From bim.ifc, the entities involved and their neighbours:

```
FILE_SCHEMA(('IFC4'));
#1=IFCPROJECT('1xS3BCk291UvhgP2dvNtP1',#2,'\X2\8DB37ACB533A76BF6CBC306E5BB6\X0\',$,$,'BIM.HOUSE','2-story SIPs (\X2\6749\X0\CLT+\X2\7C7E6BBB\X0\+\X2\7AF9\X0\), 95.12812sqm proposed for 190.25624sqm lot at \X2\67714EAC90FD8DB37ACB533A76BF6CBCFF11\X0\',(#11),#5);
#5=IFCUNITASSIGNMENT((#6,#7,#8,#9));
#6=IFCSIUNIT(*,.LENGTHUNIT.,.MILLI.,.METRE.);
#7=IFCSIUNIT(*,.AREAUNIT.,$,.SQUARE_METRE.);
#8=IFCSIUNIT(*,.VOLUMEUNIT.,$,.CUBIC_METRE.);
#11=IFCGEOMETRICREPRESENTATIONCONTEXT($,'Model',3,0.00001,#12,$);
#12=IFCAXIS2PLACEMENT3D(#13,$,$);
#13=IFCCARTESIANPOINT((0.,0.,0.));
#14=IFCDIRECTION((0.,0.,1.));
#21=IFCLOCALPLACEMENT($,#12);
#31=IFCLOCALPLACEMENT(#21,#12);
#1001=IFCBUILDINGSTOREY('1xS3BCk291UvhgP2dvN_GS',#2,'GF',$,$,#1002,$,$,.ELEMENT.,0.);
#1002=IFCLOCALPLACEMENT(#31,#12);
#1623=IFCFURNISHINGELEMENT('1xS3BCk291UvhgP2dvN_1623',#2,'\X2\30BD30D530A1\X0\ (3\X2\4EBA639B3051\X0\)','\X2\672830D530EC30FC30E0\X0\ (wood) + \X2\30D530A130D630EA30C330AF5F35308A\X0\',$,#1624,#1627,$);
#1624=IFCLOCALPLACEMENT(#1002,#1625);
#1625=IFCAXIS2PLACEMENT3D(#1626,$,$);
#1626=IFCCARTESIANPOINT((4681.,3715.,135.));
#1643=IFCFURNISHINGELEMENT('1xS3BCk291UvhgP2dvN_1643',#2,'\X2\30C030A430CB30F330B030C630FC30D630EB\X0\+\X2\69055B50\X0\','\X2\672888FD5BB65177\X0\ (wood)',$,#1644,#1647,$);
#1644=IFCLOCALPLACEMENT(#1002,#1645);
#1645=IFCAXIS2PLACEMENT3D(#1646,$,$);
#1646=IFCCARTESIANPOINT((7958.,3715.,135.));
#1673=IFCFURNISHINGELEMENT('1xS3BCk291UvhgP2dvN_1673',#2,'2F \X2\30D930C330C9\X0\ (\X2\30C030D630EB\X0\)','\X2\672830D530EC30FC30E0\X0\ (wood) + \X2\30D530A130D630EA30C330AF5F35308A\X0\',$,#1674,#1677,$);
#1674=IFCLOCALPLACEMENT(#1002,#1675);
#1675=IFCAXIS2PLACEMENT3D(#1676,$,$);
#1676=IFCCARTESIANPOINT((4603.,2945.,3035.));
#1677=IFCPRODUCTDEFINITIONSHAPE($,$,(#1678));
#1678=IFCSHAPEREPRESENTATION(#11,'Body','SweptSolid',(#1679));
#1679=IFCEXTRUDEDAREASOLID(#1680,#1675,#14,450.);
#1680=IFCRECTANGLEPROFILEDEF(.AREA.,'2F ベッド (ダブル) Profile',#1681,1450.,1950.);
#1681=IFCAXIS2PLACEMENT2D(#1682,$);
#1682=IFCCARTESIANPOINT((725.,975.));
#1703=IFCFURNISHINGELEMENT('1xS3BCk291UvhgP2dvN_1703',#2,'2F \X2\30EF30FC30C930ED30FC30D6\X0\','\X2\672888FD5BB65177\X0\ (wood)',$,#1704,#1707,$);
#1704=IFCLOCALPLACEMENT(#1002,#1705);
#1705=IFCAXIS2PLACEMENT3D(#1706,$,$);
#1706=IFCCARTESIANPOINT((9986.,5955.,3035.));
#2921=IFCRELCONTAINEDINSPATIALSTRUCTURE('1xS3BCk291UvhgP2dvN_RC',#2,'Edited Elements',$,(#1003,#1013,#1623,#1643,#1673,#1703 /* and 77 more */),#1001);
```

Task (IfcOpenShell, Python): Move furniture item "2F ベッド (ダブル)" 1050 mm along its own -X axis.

```python
import ifcopenshell
import ifcopenshell.api.geometry
import ifcopenshell.util.placement
import ifcopenshell.util.unit

model = ifcopenshell.open("bim.ifc")
unit_scale = ifcopenshell.util.unit.calculate_unit_scale(model)

item = model.by_id(1673)
matrix = ifcopenshell.util.placement.get_local_placement(item.ObjectPlacement)
matrix[:3, 3] -= matrix[:3, 0] * 1.05 / unit_scale
ifcopenshell.api.geometry.edit_object_placement(model, product=item, matrix=matrix, is_si=False)

print(ifcopenshell.util.placement.get_local_placement(item.ObjectPlacement).round(3) + 0.0)

model.write("bim-out.ifc")
```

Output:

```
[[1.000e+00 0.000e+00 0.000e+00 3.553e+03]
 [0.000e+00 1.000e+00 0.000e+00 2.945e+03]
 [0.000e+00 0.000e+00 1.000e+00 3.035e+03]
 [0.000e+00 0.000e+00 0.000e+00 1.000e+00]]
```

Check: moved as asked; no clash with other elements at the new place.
